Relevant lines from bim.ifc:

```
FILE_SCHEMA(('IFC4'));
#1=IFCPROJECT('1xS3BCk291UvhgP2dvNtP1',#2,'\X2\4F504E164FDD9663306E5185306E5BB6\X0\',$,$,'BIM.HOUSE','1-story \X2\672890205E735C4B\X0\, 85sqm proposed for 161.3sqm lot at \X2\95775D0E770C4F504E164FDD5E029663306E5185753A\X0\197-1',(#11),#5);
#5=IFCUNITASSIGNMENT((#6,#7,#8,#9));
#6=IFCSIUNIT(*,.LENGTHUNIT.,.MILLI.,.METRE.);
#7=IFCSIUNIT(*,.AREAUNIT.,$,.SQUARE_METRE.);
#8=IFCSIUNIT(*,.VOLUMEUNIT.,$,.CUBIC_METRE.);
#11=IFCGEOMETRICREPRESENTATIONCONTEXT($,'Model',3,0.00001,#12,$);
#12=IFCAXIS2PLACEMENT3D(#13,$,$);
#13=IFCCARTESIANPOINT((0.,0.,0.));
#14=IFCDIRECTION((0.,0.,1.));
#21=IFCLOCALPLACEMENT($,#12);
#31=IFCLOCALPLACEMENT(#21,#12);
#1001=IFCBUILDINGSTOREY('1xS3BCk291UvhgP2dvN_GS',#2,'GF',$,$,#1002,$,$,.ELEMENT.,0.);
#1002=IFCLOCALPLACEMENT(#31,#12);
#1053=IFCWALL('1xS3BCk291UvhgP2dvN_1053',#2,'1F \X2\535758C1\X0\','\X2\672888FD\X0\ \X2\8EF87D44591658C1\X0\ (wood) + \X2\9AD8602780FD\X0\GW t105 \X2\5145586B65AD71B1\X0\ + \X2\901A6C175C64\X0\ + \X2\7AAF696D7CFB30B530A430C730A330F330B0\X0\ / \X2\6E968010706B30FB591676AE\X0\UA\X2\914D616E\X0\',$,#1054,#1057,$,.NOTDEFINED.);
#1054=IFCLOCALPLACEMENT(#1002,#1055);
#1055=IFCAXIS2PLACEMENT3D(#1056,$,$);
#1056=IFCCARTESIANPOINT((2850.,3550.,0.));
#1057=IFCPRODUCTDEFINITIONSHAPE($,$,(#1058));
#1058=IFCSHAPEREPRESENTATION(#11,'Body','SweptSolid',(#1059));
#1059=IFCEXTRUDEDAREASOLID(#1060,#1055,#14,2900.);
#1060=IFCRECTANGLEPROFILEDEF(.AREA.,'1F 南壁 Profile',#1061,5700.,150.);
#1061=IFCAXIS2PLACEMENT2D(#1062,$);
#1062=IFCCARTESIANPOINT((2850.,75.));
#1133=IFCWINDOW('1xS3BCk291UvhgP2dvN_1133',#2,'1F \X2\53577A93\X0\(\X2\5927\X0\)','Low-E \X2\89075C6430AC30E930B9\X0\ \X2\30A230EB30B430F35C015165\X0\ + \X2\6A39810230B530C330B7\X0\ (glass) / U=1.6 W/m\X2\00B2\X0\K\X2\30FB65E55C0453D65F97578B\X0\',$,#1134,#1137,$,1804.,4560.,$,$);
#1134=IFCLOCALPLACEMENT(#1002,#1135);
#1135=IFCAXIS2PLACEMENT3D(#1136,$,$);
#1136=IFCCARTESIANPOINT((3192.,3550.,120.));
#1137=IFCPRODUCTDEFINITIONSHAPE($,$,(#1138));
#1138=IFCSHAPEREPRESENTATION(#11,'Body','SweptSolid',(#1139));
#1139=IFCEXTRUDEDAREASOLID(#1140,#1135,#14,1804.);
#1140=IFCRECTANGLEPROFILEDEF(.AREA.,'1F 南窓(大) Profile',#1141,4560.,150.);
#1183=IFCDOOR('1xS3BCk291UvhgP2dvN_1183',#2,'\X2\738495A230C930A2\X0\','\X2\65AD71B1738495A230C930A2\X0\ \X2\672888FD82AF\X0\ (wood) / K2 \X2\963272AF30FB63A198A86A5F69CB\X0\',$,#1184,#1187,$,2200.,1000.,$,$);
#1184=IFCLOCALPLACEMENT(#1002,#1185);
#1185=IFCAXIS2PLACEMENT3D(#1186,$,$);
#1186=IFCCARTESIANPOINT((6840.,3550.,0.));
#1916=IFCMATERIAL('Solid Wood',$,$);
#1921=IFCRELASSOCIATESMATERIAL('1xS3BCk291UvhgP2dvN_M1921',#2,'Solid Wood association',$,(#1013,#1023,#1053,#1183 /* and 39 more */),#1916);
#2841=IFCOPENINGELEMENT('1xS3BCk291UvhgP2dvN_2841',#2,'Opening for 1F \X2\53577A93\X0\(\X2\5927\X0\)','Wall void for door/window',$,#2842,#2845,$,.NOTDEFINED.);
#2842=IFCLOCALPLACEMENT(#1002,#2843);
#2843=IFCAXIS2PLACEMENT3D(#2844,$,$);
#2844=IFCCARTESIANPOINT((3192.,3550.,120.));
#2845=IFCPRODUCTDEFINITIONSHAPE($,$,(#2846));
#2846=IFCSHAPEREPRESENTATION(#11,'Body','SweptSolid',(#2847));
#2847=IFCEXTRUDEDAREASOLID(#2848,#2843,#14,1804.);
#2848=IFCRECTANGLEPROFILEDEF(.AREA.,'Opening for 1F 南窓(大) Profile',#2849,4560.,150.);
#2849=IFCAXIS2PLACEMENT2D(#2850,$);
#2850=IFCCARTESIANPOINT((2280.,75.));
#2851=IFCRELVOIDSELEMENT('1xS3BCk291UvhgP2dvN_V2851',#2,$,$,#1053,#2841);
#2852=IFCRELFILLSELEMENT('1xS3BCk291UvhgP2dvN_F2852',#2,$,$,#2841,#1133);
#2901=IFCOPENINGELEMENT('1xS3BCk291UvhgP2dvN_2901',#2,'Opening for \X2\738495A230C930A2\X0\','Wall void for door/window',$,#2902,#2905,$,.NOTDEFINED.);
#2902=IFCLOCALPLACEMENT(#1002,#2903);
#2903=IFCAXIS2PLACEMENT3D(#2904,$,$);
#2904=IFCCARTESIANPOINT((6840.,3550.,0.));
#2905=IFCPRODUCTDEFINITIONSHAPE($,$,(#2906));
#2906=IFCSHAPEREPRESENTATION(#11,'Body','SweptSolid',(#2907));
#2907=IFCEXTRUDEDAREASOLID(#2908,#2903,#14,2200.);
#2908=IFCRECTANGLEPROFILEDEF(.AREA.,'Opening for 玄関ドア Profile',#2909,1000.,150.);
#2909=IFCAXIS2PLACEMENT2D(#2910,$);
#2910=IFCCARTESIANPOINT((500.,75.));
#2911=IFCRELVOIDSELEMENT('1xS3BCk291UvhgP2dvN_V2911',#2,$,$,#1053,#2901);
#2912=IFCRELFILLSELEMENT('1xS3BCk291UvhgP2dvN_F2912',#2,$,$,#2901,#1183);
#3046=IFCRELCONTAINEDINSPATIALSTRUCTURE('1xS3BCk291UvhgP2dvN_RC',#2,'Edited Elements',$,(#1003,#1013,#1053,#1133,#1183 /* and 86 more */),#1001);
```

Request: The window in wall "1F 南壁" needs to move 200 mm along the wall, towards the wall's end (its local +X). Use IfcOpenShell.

```python
import ifcopenshell
import ifcopenshell.api.geometry
import ifcopenshell.util.placement
import ifcopenshell.util.unit

model = ifcopenshell.open("bim.ifc")
unit_scale = ifcopenshell.util.unit.calculate_unit_scale(model)

window = model.by_guid("1xS3BCk291UvhgP2dvN_1133")
opening = window.FillsVoids[0].RelatingOpeningElement
wall = opening.VoidsElements[0].RelatingBuildingElement

wall_matrix = ifcopenshell.util.placement.get_local_placement(wall.ObjectPlacement)
shift = wall_matrix[:3, 0] * 0.2 / unit_scale
before = ifcopenshell.util.placement.get_local_placement(window.ObjectPlacement)[:3, 3].copy()

# The window is not placed relative to its opening, so move both.
for product in (opening, window):
    matrix = ifcopenshell.util.placement.get_local_placement(product.ObjectPlacement)
    matrix[:3, 3] += shift
    ifcopenshell.api.geometry.edit_object_placement(model, product=product, matrix=matrix, is_si=False)

after = ifcopenshell.util.placement.get_local_placement(window.ObjectPlacement)[:3, 3]
print("window moved by", (after - before).round(3) + 0.0)

model.write("bim_edited.ifc")
```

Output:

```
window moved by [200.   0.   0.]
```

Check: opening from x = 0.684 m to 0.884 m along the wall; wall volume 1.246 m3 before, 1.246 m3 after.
